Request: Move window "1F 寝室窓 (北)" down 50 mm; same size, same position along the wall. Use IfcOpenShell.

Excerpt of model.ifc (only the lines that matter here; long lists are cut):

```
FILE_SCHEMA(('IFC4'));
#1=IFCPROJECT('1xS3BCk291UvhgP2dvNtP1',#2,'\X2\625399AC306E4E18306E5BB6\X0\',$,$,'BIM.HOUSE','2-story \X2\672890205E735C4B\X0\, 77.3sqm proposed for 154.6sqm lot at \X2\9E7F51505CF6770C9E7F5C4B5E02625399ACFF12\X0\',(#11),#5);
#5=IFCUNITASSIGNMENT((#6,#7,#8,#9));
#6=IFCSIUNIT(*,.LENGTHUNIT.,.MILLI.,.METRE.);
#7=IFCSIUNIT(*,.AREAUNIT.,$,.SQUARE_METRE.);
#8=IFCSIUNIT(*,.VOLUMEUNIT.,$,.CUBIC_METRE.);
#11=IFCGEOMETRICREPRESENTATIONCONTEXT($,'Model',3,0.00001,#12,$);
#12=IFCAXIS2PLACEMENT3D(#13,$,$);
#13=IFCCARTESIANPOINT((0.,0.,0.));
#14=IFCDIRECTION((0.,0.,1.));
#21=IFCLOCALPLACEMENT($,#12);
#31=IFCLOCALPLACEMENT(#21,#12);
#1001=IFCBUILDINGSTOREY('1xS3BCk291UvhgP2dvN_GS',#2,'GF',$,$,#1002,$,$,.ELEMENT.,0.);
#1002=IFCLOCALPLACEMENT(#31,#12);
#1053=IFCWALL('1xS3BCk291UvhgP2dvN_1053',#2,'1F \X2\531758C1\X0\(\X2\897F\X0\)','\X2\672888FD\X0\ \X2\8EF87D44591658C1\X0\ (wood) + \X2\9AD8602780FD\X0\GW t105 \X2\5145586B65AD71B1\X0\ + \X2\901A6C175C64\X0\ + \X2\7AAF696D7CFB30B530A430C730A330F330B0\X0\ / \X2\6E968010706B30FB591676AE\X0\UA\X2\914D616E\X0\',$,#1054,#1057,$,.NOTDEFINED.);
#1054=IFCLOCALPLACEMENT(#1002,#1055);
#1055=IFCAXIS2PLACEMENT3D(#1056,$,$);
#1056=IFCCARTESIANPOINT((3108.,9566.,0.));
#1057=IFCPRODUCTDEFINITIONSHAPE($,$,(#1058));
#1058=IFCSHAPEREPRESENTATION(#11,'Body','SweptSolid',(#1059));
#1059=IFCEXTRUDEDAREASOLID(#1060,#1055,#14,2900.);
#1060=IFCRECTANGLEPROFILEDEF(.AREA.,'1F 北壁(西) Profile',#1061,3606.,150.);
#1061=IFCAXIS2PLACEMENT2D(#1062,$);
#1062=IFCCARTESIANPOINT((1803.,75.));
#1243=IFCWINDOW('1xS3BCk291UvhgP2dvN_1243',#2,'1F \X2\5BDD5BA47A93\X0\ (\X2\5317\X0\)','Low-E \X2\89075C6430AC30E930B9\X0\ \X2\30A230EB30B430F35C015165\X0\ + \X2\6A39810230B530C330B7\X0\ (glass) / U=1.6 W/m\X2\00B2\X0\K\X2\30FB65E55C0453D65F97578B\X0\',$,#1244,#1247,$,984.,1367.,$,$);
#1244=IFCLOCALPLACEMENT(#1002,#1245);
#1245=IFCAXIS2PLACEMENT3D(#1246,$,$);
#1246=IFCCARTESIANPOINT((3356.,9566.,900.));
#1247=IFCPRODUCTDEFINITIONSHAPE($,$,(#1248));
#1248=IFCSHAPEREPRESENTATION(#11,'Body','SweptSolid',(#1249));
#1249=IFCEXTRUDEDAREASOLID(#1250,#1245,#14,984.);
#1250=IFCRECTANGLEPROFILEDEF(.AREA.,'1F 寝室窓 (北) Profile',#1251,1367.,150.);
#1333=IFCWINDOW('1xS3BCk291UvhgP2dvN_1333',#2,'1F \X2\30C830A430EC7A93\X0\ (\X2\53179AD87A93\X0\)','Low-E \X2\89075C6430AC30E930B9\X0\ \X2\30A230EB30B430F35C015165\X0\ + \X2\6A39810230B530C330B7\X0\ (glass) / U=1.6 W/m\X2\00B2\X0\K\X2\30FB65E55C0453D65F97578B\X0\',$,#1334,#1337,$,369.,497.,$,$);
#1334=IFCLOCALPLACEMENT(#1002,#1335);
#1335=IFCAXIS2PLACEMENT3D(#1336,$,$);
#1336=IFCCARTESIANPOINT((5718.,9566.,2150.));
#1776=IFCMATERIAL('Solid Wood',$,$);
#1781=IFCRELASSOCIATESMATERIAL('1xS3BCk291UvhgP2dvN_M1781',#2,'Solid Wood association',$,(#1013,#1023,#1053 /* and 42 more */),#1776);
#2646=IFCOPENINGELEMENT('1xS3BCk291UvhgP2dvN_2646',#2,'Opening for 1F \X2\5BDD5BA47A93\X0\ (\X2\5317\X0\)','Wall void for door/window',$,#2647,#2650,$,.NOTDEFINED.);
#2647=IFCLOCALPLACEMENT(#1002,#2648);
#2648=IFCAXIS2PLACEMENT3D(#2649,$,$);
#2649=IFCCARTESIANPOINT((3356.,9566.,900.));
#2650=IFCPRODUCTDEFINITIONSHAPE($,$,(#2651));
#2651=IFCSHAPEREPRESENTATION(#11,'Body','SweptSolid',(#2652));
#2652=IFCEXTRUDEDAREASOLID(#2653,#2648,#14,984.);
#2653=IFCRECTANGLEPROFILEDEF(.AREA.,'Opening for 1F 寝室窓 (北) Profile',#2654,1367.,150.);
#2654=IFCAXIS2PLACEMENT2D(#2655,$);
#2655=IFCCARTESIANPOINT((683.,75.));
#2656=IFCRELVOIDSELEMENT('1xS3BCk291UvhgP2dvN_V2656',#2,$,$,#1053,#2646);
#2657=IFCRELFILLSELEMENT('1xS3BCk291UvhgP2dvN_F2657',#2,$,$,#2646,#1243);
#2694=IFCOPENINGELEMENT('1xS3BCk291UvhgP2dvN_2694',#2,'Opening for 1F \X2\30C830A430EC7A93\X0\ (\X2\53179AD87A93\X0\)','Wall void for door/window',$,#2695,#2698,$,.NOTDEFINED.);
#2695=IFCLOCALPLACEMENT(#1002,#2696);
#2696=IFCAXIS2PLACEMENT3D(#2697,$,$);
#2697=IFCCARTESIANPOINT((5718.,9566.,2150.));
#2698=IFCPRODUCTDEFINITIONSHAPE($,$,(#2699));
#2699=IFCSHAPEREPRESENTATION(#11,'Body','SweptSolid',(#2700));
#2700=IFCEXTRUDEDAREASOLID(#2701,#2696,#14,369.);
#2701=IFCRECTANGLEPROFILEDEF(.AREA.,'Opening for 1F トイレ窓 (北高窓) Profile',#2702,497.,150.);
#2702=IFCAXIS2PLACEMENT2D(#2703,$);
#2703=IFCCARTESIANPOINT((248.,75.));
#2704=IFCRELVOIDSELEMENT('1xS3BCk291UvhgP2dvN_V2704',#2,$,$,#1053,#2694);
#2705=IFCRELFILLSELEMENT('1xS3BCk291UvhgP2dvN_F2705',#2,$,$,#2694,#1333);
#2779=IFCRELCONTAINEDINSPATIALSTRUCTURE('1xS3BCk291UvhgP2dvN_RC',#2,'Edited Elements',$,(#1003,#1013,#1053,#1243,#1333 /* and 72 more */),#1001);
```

```python
import numpy as np
import ifcopenshell
import ifcopenshell.api.geometry
import ifcopenshell.util.placement
import ifcopenshell.util.unit

model = ifcopenshell.open("model.ifc")
unit_scale = ifcopenshell.util.unit.calculate_unit_scale(model)

window = model.by_guid("1xS3BCk291UvhgP2dvN_1243")
opening = window.FillsVoids[0].RelatingOpeningElement
dz = -0.05 / unit_scale

shift = np.array([0.0, 0.0, dz])
# The window is not placed relative to its opening, so move both.
for product in (opening, window):
    matrix = ifcopenshell.util.placement.get_local_placement(product.ObjectPlacement)
    matrix[:3, 3] += shift
    ifcopenshell.api.geometry.edit_object_placement(model, product=product, matrix=matrix, is_si=False)

print(f"moved by {dz * unit_scale:+.3f} m")

model.write("model_updated.ifc")
```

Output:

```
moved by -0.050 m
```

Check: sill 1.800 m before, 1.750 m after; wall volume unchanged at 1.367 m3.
